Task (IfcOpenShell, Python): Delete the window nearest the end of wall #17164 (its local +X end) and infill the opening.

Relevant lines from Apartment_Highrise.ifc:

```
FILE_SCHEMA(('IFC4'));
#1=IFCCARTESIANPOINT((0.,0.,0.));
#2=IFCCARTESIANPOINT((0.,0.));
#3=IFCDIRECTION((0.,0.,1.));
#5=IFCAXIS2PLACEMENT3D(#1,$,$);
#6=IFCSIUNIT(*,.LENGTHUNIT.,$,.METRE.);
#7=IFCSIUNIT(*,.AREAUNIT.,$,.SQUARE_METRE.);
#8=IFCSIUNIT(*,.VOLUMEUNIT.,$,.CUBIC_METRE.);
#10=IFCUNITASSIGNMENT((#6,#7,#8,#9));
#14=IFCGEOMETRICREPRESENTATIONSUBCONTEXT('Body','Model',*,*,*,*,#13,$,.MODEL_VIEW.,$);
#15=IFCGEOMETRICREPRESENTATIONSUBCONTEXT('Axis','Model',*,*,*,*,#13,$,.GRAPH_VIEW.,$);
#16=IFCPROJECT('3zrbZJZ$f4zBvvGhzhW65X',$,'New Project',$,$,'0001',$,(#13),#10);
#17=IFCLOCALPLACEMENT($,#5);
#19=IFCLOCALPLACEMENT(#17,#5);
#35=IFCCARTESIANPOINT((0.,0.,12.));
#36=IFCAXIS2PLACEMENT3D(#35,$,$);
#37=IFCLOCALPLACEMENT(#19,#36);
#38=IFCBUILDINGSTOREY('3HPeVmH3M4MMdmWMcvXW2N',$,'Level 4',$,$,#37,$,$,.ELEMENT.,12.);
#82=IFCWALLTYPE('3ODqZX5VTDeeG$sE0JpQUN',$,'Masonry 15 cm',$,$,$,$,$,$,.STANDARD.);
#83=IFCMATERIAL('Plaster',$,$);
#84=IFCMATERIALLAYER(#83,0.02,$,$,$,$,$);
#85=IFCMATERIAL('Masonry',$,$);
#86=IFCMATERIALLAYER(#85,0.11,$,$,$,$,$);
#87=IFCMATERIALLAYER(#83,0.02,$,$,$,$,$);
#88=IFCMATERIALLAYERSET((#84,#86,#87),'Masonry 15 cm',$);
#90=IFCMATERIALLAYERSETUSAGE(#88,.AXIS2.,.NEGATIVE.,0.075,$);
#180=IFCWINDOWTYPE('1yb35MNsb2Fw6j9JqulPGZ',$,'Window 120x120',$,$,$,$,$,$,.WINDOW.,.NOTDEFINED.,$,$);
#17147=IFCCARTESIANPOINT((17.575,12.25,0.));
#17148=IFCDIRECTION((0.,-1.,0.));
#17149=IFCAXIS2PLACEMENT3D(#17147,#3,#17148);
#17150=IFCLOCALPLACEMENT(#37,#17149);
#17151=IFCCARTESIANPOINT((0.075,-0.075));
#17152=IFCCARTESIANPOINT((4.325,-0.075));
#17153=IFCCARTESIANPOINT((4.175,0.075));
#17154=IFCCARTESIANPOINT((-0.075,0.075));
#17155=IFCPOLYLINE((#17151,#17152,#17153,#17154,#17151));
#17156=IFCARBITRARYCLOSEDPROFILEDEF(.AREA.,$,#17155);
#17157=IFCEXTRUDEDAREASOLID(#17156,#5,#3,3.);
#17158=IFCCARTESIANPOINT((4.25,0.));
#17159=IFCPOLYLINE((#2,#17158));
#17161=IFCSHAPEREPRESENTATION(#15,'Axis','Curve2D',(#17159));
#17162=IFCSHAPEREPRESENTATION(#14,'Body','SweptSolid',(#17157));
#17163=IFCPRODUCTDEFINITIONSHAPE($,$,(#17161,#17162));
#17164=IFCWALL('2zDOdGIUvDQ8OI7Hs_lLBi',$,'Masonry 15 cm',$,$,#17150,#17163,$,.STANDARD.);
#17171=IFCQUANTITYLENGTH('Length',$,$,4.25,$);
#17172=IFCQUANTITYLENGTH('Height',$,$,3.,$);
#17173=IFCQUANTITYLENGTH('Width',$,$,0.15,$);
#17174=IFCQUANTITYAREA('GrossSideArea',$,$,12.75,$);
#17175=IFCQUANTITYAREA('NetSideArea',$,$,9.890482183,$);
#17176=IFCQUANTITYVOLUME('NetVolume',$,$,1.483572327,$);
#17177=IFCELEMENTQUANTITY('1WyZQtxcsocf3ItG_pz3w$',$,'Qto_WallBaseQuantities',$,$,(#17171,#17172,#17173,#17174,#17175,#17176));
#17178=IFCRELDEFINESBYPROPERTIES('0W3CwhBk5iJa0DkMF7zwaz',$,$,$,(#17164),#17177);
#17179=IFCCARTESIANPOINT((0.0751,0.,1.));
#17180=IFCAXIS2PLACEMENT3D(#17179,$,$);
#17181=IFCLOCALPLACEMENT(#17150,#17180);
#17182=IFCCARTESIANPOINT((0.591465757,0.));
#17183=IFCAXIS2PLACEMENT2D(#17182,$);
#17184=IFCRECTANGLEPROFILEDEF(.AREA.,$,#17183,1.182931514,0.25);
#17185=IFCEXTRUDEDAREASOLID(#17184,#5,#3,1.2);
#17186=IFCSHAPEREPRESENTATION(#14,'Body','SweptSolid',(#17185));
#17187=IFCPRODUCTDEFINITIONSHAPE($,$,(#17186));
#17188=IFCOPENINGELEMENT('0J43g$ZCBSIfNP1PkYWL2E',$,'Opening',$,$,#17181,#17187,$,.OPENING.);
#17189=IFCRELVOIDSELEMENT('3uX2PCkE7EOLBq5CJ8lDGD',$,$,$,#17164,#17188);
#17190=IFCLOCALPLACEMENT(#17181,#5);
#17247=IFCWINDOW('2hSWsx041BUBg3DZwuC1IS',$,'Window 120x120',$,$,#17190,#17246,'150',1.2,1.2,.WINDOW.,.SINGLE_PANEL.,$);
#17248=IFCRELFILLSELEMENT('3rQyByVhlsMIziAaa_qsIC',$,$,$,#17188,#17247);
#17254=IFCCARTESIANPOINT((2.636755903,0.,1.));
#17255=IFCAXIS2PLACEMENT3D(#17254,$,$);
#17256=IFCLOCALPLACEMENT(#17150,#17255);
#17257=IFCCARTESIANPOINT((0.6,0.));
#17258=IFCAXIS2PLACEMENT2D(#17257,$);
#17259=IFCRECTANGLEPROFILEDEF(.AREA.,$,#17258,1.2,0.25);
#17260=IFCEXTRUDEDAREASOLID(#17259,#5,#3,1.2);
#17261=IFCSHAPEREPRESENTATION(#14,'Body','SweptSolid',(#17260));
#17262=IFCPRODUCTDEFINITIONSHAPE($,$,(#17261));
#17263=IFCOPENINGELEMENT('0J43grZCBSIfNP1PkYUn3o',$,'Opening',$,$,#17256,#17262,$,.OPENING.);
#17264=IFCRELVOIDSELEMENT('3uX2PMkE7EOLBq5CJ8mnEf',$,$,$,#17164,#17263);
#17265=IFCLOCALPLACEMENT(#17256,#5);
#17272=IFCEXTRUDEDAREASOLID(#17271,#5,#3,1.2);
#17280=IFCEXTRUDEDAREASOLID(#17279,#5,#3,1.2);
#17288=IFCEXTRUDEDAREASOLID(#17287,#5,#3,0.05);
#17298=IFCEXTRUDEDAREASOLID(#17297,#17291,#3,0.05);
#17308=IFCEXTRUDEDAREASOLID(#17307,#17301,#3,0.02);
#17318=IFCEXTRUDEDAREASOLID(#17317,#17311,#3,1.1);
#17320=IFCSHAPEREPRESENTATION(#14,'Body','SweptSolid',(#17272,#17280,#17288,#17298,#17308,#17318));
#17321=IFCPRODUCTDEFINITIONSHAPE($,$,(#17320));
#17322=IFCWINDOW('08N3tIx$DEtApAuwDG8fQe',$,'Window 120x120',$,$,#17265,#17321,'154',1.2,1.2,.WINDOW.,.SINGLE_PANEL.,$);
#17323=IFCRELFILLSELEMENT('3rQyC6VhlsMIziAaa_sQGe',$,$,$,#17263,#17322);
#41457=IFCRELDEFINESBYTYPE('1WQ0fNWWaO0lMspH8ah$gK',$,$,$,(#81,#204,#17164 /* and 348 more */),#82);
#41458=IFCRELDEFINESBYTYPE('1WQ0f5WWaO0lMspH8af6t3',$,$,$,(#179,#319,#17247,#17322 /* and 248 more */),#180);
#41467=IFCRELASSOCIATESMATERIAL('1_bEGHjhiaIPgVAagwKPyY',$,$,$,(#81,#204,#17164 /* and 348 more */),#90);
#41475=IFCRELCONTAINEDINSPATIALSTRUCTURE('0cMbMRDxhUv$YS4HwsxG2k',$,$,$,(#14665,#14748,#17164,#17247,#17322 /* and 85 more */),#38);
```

```python
import ifcopenshell
import ifcopenshell.api.feature
import ifcopenshell.api.pset
import ifcopenshell.api.root
import ifcopenshell.geom
import ifcopenshell.util.element
import ifcopenshell.util.shape
import ifcopenshell.util.unit

model = ifcopenshell.open("Apartment_Highrise.ifc")
area_scale = ifcopenshell.util.unit.calculate_unit_scale(model, "AREAUNIT")
volume_scale = ifcopenshell.util.unit.calculate_unit_scale(model, "VOLUMEUNIT")
settings = ifcopenshell.geom.settings()


def volume(element):
    """Net volume in cubic metres, openings subtracted."""
    shape = ifcopenshell.geom.create_shape(settings, element)
    return ifcopenshell.util.shape.get_volume(shape.geometry)


window = model.by_guid("08N3tIx$DEtApAuwDG8fQe")
opening = window.FillsVoids[0].RelatingOpeningElement
wall = opening.VoidsElements[0].RelatingBuildingElement
before = volume(wall)

ifcopenshell.api.root.remove_product(model, product=window)
ifcopenshell.api.feature.remove_feature(model, feature=opening)

after = volume(wall)
thickness = 0.15  # wall thickness in metres

# Update the wall's stored quantities.
qto = model.by_id(ifcopenshell.util.element.get_pset(wall, "Qto_WallBaseQuantities", should_inherit=False)["id"])
ifcopenshell.api.pset.edit_qto(model, qto=qto, properties={
    "NetSideArea": after / thickness / area_scale,
    "NetVolume": after / volume_scale,
})

print(f"wall volume {before:.3f} -> {after:.3f} m3")

model.write("Apartment_Highrise-out.ifc")
```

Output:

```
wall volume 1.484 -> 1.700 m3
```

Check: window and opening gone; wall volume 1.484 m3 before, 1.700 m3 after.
